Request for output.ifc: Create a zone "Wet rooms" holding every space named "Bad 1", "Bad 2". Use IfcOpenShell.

First a look at what the model holds.

```python
import ifcopenshell

model = ifcopenshell.open("output.ifc")
print(model.schema)
seen = {}
for space in model.by_type("IfcSpace"):
    seen[space.LongName] = seen.get(space.LongName, 0) + 1
for name, count in sorted(seen.items(), key=str):
    print(count, "x", name)
print("zones:", [z.Name for z in model.by_type("IfcZone")][:20])
```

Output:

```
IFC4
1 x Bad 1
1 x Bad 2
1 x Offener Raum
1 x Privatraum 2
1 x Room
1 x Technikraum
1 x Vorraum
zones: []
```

```python
import ifcopenshell
import ifcopenshell.api.group
import ifcopenshell.api.root

model = ifcopenshell.open("output.ifc")

names = {"Bad 1", "Bad 2"}
spaces = [s for s in model.by_type("IfcSpace") if s.LongName in names]

zone = ifcopenshell.api.root.create_entity(model, ifc_class="IfcZone", name="Wet rooms")
ifcopenshell.api.group.assign_group(model, products=spaces, group=zone)
print(len(spaces), "spaces in", zone.Name)

model.write("output-out.ifc")
```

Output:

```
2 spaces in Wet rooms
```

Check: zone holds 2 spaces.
